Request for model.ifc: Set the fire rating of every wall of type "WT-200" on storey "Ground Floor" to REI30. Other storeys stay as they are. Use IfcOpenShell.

First a look at what the model holds.

```python
import ifcopenshell
import ifcopenshell.util.element

model = ifcopenshell.open("model.ifc")
print(model.schema)
storey = next(s for s in model.by_type("IfcBuildingStorey") if s.Name == "Ground Floor")
walls = [e for e in ifcopenshell.util.element.get_decomposition(storey) if e.is_a("IfcWall")]
seen = {}
for e in walls:
    element_type = ifcopenshell.util.element.get_type(e)
    key = (element_type.Name if element_type != e and element_type else None, ifcopenshell.util.element.get_pset(e, "Pset_WallCommon", "FireRating"))
    seen[key] = seen.get(key, 0) + 1
for (name, value), count in sorted(seen.items(), key=str):
    print(count, "x", name, "|", value)
```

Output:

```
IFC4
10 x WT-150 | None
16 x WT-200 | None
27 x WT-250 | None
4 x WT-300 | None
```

```python
import ifcopenshell
import ifcopenshell.api.pset
import ifcopenshell.util.element

model = ifcopenshell.open("model.ifc")

storey = next(s for s in model.by_type("IfcBuildingStorey") if s.Name == "Ground Floor")
walls = [e for e in ifcopenshell.util.element.get_decomposition(storey) if e.is_a("IfcWall")]

count = 0
for e in walls:
    element_type = ifcopenshell.util.element.get_type(e)
    if element_type in (None, e) or element_type.Name != "WT-200":
        continue
    # add_pset returns the element's existing set when there is one.
    pset = ifcopenshell.api.pset.add_pset(model, product=e, name="Pset_WallCommon")
    ifcopenshell.api.pset.edit_pset(model, pset=pset, properties={"FireRating": "REI30"})
    count += 1

print(count, "walls updated")

model.write("model_updated.ifc")
```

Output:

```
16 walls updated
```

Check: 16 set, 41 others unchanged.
